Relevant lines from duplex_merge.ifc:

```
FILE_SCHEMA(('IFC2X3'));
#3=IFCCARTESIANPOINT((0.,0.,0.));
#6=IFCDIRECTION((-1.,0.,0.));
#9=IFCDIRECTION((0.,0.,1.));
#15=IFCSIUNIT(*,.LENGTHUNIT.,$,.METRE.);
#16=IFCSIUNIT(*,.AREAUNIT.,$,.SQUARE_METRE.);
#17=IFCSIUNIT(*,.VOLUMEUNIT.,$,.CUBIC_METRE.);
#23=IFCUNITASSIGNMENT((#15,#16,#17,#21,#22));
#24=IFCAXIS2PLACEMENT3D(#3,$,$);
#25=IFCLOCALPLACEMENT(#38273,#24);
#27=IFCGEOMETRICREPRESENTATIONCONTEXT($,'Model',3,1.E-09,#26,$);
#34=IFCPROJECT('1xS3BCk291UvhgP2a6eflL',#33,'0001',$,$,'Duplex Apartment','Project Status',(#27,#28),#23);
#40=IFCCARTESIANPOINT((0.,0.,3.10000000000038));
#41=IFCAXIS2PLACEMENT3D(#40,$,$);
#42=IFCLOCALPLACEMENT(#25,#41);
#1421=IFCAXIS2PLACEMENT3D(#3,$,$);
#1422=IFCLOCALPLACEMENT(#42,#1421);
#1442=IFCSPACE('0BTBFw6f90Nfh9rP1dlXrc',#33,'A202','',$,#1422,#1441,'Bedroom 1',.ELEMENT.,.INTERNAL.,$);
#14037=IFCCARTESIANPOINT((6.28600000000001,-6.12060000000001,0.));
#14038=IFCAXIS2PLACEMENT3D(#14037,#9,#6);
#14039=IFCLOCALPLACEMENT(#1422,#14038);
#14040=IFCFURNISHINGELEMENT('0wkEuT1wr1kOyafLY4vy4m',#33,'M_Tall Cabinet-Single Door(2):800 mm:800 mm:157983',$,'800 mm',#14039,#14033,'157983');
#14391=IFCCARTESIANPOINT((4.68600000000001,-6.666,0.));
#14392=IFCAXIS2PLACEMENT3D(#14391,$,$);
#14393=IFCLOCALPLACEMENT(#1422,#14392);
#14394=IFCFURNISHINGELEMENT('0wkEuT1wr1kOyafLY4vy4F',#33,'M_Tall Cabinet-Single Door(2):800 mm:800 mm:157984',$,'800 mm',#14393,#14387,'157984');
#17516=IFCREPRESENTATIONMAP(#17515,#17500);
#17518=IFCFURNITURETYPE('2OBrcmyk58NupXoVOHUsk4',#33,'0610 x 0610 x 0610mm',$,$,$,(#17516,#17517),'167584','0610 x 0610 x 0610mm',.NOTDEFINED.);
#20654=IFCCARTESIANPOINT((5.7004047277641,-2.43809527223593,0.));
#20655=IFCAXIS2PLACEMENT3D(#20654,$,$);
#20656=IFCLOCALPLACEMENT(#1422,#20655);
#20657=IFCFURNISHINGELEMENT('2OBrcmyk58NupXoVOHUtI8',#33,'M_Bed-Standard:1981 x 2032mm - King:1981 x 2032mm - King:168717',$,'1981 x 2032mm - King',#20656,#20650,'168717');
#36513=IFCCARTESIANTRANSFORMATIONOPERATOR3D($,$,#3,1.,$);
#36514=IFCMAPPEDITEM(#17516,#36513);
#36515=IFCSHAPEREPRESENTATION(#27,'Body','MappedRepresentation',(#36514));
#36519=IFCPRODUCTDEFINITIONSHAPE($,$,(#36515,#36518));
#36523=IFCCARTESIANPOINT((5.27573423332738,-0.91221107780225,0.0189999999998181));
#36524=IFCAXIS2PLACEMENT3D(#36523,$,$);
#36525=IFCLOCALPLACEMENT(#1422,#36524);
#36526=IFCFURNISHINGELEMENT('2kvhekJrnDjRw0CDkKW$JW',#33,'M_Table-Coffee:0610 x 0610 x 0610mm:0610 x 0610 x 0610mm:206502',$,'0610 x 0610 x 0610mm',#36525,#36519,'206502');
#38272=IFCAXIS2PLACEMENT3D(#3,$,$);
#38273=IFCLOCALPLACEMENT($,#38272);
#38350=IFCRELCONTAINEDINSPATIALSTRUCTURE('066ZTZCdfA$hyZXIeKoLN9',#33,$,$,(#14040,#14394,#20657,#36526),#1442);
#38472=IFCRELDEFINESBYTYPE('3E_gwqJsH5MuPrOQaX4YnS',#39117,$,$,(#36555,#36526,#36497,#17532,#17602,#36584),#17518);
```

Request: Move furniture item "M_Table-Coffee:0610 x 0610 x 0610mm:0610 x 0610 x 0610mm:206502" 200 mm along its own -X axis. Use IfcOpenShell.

```python
import ifcopenshell
import ifcopenshell.api.geometry
import ifcopenshell.util.placement

model = ifcopenshell.open("duplex_merge.ifc")

item = model.by_guid("2kvhekJrnDjRw0CDkKW$JW")
matrix = ifcopenshell.util.placement.get_local_placement(item.ObjectPlacement)
matrix[:3, 3] -= matrix[:3, 0] * 0.2
ifcopenshell.api.geometry.edit_object_placement(model, product=item, matrix=matrix, is_si=False)

print(ifcopenshell.util.placement.get_local_placement(item.ObjectPlacement).round(3) + 0.0)

model.write("duplex_merge_v2.ifc")
```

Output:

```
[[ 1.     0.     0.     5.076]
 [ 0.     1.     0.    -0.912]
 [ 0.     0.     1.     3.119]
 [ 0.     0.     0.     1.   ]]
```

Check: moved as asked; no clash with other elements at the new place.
